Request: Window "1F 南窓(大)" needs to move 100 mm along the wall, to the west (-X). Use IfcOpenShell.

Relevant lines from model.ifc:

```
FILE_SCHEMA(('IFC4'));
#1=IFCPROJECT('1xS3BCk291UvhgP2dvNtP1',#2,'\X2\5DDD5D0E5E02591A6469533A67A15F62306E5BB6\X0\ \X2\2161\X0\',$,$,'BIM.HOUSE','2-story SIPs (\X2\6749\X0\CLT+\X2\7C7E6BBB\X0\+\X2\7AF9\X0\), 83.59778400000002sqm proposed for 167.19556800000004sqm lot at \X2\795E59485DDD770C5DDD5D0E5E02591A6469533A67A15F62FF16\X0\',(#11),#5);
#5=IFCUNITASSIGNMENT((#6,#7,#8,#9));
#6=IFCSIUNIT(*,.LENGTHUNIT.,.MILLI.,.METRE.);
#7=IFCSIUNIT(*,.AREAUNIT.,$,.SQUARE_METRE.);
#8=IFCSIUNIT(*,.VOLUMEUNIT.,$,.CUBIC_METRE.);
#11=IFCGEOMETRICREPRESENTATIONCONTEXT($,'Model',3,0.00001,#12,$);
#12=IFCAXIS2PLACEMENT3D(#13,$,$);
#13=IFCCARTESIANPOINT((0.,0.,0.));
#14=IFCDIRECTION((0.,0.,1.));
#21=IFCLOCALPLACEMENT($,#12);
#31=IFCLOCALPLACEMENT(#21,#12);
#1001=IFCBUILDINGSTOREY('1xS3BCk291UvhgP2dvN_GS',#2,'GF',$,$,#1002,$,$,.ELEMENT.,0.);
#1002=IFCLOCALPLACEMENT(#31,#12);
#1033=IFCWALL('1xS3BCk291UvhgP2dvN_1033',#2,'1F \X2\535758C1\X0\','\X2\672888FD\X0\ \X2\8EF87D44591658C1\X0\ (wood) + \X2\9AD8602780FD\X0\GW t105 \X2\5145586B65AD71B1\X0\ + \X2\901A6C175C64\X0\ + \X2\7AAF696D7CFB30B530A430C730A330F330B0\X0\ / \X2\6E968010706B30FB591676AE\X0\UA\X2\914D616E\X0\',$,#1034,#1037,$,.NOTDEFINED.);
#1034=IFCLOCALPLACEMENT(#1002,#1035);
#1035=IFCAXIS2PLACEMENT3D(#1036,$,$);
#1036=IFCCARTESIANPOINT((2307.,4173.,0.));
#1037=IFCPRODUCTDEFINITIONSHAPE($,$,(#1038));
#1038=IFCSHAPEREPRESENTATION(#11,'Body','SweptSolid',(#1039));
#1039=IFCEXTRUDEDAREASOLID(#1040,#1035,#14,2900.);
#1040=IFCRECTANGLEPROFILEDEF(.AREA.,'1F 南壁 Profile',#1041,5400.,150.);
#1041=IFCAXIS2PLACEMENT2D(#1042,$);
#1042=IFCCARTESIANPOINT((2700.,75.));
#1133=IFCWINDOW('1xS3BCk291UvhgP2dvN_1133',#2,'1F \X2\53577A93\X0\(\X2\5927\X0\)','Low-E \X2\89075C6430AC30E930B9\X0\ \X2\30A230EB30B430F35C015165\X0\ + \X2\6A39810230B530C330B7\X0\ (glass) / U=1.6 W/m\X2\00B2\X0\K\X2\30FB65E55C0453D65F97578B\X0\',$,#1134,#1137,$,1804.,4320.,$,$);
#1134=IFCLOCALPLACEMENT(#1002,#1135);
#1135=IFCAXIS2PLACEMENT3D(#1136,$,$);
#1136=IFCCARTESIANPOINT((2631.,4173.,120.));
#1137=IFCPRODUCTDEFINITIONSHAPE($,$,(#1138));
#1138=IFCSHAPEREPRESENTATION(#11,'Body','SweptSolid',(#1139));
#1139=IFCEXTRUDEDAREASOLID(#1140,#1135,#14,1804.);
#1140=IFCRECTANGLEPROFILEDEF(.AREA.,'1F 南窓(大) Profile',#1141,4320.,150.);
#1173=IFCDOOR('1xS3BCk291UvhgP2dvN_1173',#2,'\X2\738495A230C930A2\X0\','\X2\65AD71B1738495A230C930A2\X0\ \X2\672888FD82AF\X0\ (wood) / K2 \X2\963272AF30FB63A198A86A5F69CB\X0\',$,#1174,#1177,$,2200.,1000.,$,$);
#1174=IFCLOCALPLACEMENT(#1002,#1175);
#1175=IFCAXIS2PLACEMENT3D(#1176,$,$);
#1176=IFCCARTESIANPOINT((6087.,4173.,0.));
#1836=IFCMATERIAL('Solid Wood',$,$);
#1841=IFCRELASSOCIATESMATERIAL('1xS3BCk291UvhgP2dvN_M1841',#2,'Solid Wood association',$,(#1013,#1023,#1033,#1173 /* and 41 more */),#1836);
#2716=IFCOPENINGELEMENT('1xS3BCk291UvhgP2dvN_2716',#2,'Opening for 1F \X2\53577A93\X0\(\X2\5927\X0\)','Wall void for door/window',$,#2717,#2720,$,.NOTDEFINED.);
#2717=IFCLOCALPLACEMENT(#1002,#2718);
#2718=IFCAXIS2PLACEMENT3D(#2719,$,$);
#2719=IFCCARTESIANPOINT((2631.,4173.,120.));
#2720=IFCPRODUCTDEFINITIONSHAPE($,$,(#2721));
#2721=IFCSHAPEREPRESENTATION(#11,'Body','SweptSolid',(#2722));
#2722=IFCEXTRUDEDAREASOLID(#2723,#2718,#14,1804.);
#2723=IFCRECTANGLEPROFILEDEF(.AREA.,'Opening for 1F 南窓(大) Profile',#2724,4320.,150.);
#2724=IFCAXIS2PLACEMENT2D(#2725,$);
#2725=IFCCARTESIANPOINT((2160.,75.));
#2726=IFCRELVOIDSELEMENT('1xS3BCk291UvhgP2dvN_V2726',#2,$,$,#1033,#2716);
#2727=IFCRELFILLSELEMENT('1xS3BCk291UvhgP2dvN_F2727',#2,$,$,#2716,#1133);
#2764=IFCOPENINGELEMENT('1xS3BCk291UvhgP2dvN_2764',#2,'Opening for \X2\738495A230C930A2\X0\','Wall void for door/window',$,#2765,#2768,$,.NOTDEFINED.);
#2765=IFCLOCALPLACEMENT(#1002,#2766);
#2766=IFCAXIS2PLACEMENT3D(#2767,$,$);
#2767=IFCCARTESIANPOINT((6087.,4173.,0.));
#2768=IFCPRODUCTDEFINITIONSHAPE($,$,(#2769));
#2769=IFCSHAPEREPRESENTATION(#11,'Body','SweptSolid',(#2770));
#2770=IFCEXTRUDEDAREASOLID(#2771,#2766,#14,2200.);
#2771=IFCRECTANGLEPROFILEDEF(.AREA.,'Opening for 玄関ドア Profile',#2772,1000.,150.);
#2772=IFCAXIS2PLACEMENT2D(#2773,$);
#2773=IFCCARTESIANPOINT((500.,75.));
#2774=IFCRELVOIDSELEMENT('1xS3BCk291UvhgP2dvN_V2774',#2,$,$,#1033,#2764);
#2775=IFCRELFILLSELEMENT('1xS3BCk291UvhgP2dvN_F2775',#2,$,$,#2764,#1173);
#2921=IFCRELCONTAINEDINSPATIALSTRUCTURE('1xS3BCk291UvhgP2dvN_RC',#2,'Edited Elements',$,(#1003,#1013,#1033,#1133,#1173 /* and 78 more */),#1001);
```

```python
import ifcopenshell
import ifcopenshell.api.geometry
import ifcopenshell.util.placement

model = ifcopenshell.open("model.ifc")

window = model.by_id(1133)
opening = window.FillsVoids[0].RelatingOpeningElement
wall = opening.VoidsElements[0].RelatingBuildingElement

wall_matrix = ifcopenshell.util.placement.get_local_placement(wall.ObjectPlacement)
shift = wall_matrix[:3, 0] * -100.0
before = ifcopenshell.util.placement.get_local_placement(window.ObjectPlacement)[:3, 3].copy()

# The window is not placed relative to its opening, so move both.
for product in (opening, window):
    matrix = ifcopenshell.util.placement.get_local_placement(product.ObjectPlacement)
    matrix[:3, 3] += shift
    ifcopenshell.api.geometry.edit_object_placement(model, product=product, matrix=matrix, is_si=False)

after = ifcopenshell.util.placement.get_local_placement(window.ObjectPlacement)[:3, 3]
print("window moved by", (after - before).round(3) + 0.0)

model.write("model_v2.ifc")
```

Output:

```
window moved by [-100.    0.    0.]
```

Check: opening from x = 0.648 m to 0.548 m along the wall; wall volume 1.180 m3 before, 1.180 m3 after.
